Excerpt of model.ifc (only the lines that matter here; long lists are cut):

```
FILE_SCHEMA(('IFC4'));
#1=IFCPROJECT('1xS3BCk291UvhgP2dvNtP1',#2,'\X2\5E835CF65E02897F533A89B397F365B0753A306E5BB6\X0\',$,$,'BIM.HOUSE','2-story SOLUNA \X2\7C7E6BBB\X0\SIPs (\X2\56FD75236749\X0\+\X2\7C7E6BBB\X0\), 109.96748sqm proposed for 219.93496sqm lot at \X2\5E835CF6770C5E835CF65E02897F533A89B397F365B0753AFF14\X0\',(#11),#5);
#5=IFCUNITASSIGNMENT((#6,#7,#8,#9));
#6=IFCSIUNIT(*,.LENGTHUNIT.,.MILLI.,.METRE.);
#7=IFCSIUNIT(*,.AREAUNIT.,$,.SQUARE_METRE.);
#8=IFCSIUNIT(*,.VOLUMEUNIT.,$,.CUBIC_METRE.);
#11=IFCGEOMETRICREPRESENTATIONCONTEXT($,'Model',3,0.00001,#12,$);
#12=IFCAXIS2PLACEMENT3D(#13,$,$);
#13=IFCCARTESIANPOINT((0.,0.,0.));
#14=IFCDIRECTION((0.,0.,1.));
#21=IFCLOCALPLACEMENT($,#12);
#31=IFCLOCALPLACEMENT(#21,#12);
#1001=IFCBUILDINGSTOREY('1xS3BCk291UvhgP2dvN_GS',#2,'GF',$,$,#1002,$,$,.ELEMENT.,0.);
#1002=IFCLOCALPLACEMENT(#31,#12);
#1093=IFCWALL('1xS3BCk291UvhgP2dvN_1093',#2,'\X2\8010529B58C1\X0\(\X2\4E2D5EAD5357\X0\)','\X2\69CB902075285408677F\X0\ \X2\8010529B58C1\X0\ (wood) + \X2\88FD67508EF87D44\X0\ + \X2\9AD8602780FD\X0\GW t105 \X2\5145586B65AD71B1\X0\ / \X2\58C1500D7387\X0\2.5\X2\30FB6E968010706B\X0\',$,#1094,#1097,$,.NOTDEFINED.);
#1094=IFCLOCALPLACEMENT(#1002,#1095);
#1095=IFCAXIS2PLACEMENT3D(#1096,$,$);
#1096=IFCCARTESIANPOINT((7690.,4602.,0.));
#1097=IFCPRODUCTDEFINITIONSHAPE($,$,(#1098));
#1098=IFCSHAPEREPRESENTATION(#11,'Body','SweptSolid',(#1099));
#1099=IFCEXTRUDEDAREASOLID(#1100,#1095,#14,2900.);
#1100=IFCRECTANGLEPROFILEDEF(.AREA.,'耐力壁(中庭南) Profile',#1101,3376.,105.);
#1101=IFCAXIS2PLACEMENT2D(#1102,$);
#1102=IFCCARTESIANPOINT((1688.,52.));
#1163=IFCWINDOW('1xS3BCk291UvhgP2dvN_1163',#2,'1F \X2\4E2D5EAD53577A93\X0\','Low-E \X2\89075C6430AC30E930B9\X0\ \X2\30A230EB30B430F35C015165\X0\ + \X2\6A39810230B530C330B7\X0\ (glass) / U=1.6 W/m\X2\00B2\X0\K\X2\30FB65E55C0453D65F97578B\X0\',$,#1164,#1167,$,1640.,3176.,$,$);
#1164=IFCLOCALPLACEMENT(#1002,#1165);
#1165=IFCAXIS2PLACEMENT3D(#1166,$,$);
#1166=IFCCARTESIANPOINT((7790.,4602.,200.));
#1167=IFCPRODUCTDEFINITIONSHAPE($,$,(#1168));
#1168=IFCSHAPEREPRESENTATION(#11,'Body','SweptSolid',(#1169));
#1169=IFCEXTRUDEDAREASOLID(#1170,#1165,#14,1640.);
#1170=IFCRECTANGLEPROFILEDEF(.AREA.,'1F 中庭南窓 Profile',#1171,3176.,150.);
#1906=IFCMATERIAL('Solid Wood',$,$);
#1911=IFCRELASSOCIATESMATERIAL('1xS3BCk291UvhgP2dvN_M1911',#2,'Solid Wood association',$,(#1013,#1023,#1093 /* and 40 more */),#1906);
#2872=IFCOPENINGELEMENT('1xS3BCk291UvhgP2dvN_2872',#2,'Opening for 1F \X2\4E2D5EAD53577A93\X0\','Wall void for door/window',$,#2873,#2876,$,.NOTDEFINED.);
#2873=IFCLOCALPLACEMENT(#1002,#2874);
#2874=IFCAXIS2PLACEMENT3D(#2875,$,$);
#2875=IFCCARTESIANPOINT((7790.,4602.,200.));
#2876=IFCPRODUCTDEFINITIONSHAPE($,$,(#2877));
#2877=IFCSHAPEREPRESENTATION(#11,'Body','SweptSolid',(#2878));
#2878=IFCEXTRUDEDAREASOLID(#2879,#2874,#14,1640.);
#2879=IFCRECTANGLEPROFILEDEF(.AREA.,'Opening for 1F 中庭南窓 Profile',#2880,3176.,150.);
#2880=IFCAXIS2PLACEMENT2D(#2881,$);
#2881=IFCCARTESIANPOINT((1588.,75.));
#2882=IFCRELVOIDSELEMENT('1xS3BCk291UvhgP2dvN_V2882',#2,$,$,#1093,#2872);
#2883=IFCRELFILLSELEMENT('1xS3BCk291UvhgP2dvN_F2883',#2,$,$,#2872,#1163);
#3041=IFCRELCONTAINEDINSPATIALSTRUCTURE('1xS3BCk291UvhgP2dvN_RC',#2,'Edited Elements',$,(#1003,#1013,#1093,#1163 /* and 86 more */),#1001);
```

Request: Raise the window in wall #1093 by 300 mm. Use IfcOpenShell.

```python
import numpy as np
import ifcopenshell
import ifcopenshell.api.geometry
import ifcopenshell.util.placement
import ifcopenshell.util.unit

model = ifcopenshell.open("model.ifc")
unit_scale = ifcopenshell.util.unit.calculate_unit_scale(model)

window = model.by_guid("1xS3BCk291UvhgP2dvN_1163")
opening = window.FillsVoids[0].RelatingOpeningElement
dz = 0.3 / unit_scale

shift = np.array([0.0, 0.0, dz])
# The window is not placed relative to its opening, so move both.
for product in (opening, window):
    matrix = ifcopenshell.util.placement.get_local_placement(product.ObjectPlacement)
    matrix[:3, 3] += shift
    ifcopenshell.api.geometry.edit_object_placement(model, product=product, matrix=matrix, is_si=False)

print(f"moved by {dz * unit_scale:+.3f} m")

model.write("model_updated.ifc")
```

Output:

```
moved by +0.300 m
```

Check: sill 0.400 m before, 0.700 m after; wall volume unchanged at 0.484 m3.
